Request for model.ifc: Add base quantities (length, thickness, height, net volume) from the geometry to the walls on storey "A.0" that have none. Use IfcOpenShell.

First a look at what the model holds.

```python
import ifcopenshell
import ifcopenshell.util.element
import ifcopenshell.util.unit

model = ifcopenshell.open("model.ifc")
print(model.schema)
for unit_type in ("LENGTHUNIT", "AREAUNIT", "VOLUMEUNIT"):
    print(unit_type, ifcopenshell.util.unit.calculate_unit_scale(model, unit_type))
storey = next(s for s in model.by_type("IfcBuildingStorey") if s.Name == "A.0")
walls = [e for e in ifcopenshell.util.element.get_decomposition(storey) if e.is_a("IfcWall")]
for e in sorted(walls, key=lambda e: e.id()):
    print(e.id(), e.is_a(), e.Name, list(ifcopenshell.util.element.get_psets(e, qtos_only=True)), sep=" | ")
```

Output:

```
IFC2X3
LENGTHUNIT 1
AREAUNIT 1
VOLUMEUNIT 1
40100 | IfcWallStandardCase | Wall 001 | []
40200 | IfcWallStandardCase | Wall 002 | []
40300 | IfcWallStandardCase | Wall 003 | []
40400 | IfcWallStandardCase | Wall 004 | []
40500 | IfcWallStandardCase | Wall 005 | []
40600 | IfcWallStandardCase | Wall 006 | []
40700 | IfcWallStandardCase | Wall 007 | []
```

```python
import ifcopenshell
import ifcopenshell.api.pset
import ifcopenshell.geom
import ifcopenshell.util.element
import ifcopenshell.util.shape
import ifcopenshell.util.unit

model = ifcopenshell.open("model.ifc")
unit_scale = ifcopenshell.util.unit.calculate_unit_scale(model)
volume_scale = ifcopenshell.util.unit.calculate_unit_scale(model, "VOLUMEUNIT")
settings = ifcopenshell.geom.settings()

storey = next(s for s in model.by_type("IfcBuildingStorey") if s.Name == "A.0")
walls = [e for e in ifcopenshell.util.element.get_decomposition(storey) if e.is_a("IfcWall")]

for e in sorted(walls, key=lambda e: e.id()):
    if ifcopenshell.util.element.get_psets(e, qtos_only=True, should_inherit=False):
        continue
    # Geometry comes back in metres, in the element's own axes.
    shape = ifcopenshell.geom.create_shape(settings, e)
    values = {
        "Length": ifcopenshell.util.shape.get_x(shape.geometry) / unit_scale,
        "Width": ifcopenshell.util.shape.get_y(shape.geometry) / unit_scale,
        "Height": ifcopenshell.util.shape.get_z(shape.geometry) / unit_scale,
        "NetVolume": ifcopenshell.util.shape.get_volume(shape.geometry) / volume_scale,
    }
    qto = ifcopenshell.api.pset.add_qto(model, product=e, name="BaseQuantities")
    ifcopenshell.api.pset.edit_qto(model, qto=qto, properties=values)
    print(e.id(), {k: round(v, 3) for k, v in values.items()})

model.write("model_updated.ifc")
```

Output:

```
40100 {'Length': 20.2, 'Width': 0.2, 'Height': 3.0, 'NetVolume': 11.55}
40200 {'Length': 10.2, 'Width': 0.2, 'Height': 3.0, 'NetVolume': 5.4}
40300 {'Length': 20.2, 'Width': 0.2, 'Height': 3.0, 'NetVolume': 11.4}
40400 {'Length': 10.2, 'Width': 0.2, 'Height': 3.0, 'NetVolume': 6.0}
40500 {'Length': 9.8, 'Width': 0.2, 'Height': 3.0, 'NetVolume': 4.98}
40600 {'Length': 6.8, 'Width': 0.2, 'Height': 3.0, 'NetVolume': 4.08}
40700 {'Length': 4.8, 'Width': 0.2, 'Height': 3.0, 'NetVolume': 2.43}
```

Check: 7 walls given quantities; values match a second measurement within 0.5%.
